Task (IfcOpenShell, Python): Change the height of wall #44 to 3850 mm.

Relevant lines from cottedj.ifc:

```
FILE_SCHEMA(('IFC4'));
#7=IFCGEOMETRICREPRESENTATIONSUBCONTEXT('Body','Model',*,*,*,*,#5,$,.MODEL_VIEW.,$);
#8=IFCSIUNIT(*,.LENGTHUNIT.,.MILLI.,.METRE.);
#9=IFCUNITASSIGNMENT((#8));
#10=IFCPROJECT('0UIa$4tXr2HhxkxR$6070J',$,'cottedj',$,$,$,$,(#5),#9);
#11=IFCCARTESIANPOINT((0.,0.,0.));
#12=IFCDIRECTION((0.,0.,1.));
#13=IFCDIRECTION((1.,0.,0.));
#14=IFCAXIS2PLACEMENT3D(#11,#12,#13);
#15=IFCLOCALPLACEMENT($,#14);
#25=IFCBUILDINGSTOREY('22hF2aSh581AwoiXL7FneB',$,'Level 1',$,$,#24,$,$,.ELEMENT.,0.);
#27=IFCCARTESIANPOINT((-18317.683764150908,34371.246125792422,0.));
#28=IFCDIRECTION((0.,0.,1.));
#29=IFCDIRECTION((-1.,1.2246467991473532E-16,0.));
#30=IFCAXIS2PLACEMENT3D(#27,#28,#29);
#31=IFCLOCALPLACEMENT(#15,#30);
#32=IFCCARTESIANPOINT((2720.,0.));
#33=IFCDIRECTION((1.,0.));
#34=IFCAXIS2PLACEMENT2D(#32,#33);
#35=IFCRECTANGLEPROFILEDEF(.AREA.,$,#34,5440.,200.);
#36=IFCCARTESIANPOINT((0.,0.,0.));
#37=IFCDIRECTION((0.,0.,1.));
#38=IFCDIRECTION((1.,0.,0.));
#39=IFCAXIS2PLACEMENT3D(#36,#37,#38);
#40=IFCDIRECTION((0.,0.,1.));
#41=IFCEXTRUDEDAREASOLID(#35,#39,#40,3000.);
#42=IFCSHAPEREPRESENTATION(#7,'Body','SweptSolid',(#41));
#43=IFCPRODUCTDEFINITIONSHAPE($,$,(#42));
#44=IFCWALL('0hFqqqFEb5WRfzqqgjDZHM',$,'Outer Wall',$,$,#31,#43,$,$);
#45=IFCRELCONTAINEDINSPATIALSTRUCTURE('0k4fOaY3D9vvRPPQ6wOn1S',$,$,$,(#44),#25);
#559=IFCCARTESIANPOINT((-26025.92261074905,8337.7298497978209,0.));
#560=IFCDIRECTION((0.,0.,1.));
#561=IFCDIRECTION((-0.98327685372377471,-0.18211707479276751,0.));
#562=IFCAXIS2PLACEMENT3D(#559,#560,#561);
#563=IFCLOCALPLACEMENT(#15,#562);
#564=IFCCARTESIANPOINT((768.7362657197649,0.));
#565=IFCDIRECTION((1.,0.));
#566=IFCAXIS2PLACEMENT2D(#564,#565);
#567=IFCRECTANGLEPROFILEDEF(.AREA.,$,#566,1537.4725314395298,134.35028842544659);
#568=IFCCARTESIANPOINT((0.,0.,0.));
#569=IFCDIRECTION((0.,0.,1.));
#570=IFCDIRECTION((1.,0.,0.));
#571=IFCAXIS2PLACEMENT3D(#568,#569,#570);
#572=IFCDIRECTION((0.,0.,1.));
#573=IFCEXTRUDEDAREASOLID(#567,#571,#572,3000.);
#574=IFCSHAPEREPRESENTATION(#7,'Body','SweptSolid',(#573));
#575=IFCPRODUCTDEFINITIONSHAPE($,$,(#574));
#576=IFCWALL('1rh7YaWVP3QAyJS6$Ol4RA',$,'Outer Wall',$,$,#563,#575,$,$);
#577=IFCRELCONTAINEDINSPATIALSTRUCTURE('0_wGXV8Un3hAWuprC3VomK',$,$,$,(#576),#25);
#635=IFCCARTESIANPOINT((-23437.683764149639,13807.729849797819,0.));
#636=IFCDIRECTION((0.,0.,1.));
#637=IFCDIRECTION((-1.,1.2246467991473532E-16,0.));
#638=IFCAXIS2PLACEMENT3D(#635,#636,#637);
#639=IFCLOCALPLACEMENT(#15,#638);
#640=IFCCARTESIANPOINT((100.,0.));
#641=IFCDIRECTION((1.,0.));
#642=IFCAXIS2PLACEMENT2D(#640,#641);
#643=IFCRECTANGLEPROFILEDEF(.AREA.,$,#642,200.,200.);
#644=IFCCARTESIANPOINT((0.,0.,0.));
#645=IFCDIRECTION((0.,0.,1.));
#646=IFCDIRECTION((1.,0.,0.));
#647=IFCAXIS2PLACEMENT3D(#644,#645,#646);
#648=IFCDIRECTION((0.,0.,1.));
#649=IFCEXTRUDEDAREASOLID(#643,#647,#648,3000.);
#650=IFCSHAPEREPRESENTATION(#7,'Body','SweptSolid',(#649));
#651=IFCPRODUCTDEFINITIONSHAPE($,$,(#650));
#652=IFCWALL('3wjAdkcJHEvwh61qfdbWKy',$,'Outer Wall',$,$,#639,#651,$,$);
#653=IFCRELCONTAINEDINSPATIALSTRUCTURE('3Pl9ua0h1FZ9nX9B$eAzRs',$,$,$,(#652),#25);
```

```python
import ifcopenshell
import ifcopenshell.geom
import ifcopenshell.util.representation
import ifcopenshell.util.shape

model = ifcopenshell.open("cottedj.ifc")
settings = ifcopenshell.geom.settings()


def volume(element):
    """Net volume in cubic metres, openings subtracted."""
    shape = ifcopenshell.geom.create_shape(settings, element)
    return ifcopenshell.util.shape.get_volume(shape.geometry)


wall = model.by_guid("0hFqqqFEb5WRfzqqgjDZHM")
before = volume(wall)

body = ifcopenshell.util.representation.get_representation(wall, "Model", "Body")
solid = body.Items[0]
old_height = solid.Depth
solid.Depth = 3850.0
after = volume(wall)

print(f"height {old_height:g} -> {solid.Depth:g}, volume {before:.3f} -> {after:.3f} m3")

model.write("cottedj_edited.ifc")
```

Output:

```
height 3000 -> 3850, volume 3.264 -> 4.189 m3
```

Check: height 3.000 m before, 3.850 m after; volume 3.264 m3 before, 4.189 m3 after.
